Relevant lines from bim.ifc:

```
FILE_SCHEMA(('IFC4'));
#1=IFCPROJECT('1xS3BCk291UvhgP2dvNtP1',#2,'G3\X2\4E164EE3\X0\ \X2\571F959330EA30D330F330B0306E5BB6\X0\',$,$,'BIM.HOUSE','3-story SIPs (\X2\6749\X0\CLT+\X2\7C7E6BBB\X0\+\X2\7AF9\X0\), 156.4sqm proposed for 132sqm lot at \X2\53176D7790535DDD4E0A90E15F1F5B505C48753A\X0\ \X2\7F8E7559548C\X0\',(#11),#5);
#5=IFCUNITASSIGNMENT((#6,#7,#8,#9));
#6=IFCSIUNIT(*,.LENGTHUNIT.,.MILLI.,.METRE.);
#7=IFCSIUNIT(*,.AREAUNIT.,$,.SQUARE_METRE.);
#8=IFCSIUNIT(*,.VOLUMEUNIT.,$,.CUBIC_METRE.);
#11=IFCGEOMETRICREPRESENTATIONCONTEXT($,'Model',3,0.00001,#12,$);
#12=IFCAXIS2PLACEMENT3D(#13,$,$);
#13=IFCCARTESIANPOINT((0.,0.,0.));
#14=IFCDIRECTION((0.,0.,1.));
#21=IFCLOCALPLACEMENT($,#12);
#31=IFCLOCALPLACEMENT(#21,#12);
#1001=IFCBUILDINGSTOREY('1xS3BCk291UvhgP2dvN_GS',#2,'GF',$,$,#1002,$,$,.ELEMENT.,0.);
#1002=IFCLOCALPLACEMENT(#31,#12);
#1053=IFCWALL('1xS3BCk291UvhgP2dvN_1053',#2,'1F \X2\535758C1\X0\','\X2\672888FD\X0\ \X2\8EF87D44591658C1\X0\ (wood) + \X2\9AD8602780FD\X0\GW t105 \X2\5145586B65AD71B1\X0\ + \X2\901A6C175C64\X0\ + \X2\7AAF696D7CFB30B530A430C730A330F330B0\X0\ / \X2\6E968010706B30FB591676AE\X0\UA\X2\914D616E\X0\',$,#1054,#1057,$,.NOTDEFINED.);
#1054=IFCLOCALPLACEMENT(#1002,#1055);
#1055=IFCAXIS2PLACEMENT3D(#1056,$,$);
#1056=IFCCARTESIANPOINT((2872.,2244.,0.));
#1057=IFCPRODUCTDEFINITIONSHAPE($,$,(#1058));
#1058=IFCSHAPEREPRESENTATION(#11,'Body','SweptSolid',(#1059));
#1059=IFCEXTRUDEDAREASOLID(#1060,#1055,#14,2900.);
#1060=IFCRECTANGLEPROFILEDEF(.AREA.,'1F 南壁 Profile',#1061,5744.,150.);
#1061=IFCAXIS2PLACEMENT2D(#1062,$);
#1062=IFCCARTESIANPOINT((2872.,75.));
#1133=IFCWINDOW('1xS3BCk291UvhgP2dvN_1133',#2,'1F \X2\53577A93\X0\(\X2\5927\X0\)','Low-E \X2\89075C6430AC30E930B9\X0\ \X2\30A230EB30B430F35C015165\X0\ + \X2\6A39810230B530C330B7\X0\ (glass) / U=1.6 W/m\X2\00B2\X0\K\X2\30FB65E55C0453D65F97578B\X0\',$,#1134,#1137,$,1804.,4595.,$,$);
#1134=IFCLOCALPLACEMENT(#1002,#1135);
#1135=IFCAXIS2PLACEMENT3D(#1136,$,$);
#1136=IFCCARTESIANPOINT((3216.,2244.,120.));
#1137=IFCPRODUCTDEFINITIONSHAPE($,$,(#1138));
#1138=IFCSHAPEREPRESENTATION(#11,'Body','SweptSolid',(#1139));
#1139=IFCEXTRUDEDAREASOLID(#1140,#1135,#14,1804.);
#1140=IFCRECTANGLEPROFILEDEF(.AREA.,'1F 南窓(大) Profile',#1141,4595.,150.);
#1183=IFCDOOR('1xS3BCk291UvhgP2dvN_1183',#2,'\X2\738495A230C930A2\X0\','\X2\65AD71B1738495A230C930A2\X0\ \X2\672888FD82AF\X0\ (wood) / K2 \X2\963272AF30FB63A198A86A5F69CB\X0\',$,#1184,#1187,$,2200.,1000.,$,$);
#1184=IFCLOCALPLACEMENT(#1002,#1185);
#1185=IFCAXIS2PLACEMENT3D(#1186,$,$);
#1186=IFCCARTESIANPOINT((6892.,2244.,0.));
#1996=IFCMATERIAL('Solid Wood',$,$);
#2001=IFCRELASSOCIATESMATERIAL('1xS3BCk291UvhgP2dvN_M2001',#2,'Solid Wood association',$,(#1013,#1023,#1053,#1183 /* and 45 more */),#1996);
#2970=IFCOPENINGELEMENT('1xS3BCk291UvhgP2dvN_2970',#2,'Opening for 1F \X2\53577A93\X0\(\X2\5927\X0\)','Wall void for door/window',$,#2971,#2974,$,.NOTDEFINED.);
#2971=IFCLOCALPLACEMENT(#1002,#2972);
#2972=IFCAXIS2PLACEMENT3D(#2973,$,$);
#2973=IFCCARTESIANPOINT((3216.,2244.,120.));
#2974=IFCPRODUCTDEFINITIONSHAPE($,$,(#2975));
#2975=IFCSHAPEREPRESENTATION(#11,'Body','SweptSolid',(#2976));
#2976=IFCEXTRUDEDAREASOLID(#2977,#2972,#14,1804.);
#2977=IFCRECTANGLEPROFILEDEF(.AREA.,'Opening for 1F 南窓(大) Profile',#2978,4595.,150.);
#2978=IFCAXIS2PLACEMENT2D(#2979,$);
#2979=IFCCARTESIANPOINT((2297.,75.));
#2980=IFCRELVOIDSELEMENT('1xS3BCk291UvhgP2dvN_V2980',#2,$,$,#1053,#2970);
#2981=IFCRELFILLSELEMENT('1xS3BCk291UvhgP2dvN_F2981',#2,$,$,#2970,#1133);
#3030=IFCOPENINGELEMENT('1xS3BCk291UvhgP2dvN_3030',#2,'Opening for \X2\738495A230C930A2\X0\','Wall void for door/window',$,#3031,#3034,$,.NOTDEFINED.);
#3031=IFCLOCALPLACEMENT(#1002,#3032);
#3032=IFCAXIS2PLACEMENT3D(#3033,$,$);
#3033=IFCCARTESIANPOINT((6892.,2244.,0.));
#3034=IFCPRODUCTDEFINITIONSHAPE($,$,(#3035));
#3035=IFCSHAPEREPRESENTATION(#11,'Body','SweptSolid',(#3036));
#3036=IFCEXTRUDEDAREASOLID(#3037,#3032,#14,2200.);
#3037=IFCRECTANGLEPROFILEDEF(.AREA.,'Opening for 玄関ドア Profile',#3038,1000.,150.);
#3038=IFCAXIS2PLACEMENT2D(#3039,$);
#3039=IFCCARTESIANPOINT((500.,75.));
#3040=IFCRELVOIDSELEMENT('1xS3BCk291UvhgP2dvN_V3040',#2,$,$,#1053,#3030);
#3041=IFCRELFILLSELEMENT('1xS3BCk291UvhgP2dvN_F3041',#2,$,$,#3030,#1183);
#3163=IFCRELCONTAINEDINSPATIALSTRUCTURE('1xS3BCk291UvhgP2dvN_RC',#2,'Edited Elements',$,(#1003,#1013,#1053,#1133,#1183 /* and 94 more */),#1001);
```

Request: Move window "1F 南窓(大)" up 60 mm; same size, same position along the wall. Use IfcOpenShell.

```python
import numpy as np
import ifcopenshell
import ifcopenshell.api.geometry
import ifcopenshell.util.placement
import ifcopenshell.util.unit

model = ifcopenshell.open("bim.ifc")
unit_scale = ifcopenshell.util.unit.calculate_unit_scale(model)

window = model.by_id(1133)
opening = window.FillsVoids[0].RelatingOpeningElement
dz = 60.0

shift = np.array([0.0, 0.0, dz])
# The window is not placed relative to its opening, so move both.
for product in (opening, window):
    matrix = ifcopenshell.util.placement.get_local_placement(product.ObjectPlacement)
    matrix[:3, 3] += shift
    ifcopenshell.api.geometry.edit_object_placement(model, product=product, matrix=matrix, is_si=False)

print(f"moved by {dz * unit_scale:+.3f} m")

model.write("bim-out.ifc")
```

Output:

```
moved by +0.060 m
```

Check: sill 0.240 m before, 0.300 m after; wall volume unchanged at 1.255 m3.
